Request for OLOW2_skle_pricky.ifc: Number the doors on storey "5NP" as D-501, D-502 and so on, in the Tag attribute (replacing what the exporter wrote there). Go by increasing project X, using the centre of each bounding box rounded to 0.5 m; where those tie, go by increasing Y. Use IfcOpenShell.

First a look at what the model holds.

```python
import ifcopenshell
import ifcopenshell.util.element
import ifcopenshell.util.placement

model = ifcopenshell.open("OLOW2_skle_pricky.ifc")
print(model.schema)
storey = next(s for s in model.by_type("IfcBuildingStorey") if s.Name == "5NP")
doors = [e for e in ifcopenshell.util.element.get_decomposition(storey) if e.is_a("IfcDoor")]
for e in sorted(doors, key=lambda e: e.id()):
    origin = ifcopenshell.util.placement.get_local_placement(e.ObjectPlacement)[:3, 3]
    print(e.id(), e.Tag, e.Name, origin.round(2) + 0.0, sep=" | ")
```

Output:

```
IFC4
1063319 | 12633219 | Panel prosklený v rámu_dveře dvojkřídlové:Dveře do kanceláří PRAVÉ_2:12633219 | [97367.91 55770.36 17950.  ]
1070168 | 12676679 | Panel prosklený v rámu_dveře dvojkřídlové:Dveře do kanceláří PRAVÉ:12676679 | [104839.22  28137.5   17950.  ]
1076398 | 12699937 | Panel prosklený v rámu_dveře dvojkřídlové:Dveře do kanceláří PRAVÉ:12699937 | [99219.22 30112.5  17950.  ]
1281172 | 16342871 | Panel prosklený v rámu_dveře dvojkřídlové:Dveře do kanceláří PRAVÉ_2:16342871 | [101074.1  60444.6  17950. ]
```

```python
import ifcopenshell
import ifcopenshell.geom
import ifcopenshell.util.element
import ifcopenshell.util.shape

model = ifcopenshell.open("OLOW2_skle_pricky.ifc")
settings = ifcopenshell.geom.settings()
settings.set("use-world-coords", True)


def centre(element):
    shape = ifcopenshell.geom.create_shape(settings, element)
    return ifcopenshell.util.shape.get_bbox_centroid(shape.geometry)


storey = next(s for s in model.by_type("IfcBuildingStorey") if s.Name == "5NP")
doors = [e for e in ifcopenshell.util.element.get_decomposition(storey) if e.is_a("IfcDoor")]

# Insertion points can sit at a corner or the storey origin, so sort by the geometry (in metres).
centres = {e: centre(e) for e in doors}
doors.sort(key=lambda e: (round(centres[e][0] / 0.5), centres[e][1]))

for i, e in enumerate(doors, start=1):
    number = f"D-5{i:02d}"
    e.Tag = number
    print(e.id(), number)

model.write("OLOW2_skle_pricky-out.ifc")
```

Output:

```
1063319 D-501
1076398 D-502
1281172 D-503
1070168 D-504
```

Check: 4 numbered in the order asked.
